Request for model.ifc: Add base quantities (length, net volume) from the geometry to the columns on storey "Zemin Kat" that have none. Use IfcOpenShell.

First a look at what the model holds.

```python
import ifcopenshell
import ifcopenshell.util.element
import ifcopenshell.util.unit

model = ifcopenshell.open("model.ifc")
print(model.schema)
for unit_type in ("LENGTHUNIT", "AREAUNIT", "VOLUMEUNIT"):
    print(unit_type, ifcopenshell.util.unit.calculate_unit_scale(model, unit_type))
storey = next(s for s in model.by_type("IfcBuildingStorey") if s.Name == "Zemin Kat")
columns = [e for e in ifcopenshell.util.element.get_decomposition(storey) if e.is_a("IfcColumn")]
for e in sorted(columns, key=lambda e: e.id()):
    print(e.id(), e.is_a(), e.Name, list(ifcopenshell.util.element.get_psets(e, qtos_only=True)), sep=" | ")
```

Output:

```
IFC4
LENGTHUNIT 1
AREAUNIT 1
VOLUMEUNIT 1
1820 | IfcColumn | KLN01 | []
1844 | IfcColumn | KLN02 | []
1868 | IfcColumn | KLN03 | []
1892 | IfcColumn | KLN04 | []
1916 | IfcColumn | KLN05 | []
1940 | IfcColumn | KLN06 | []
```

```python
import ifcopenshell
import ifcopenshell.api.pset
import ifcopenshell.geom
import ifcopenshell.util.element
import ifcopenshell.util.shape
import ifcopenshell.util.unit

model = ifcopenshell.open("model.ifc")
unit_scale = ifcopenshell.util.unit.calculate_unit_scale(model)
volume_scale = ifcopenshell.util.unit.calculate_unit_scale(model, "VOLUMEUNIT")
settings = ifcopenshell.geom.settings()

storey = next(s for s in model.by_type("IfcBuildingStorey") if s.Name == "Zemin Kat")
columns = [e for e in ifcopenshell.util.element.get_decomposition(storey) if e.is_a("IfcColumn")]

for e in sorted(columns, key=lambda e: e.id()):
    if ifcopenshell.util.element.get_psets(e, qtos_only=True, should_inherit=False):
        continue
    # Geometry comes back in metres, in the element's own axes.
    shape = ifcopenshell.geom.create_shape(settings, e)
    values = {
        "Length": ifcopenshell.util.shape.get_z(shape.geometry) / unit_scale,
        "NetVolume": ifcopenshell.util.shape.get_volume(shape.geometry) / volume_scale,
    }
    qto = ifcopenshell.api.pset.add_qto(model, product=e, name="Qto_ColumnBaseQuantities")
    ifcopenshell.api.pset.edit_qto(model, qto=qto, properties=values)
    print(e.id(), {k: round(v, 3) for k, v in values.items()})

model.write("model-out.ifc")
```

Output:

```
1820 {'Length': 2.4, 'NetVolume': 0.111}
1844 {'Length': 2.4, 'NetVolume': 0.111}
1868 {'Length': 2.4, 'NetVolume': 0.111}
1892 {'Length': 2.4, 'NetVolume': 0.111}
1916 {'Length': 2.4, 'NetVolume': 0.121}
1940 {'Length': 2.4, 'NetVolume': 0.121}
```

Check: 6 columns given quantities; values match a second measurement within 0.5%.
